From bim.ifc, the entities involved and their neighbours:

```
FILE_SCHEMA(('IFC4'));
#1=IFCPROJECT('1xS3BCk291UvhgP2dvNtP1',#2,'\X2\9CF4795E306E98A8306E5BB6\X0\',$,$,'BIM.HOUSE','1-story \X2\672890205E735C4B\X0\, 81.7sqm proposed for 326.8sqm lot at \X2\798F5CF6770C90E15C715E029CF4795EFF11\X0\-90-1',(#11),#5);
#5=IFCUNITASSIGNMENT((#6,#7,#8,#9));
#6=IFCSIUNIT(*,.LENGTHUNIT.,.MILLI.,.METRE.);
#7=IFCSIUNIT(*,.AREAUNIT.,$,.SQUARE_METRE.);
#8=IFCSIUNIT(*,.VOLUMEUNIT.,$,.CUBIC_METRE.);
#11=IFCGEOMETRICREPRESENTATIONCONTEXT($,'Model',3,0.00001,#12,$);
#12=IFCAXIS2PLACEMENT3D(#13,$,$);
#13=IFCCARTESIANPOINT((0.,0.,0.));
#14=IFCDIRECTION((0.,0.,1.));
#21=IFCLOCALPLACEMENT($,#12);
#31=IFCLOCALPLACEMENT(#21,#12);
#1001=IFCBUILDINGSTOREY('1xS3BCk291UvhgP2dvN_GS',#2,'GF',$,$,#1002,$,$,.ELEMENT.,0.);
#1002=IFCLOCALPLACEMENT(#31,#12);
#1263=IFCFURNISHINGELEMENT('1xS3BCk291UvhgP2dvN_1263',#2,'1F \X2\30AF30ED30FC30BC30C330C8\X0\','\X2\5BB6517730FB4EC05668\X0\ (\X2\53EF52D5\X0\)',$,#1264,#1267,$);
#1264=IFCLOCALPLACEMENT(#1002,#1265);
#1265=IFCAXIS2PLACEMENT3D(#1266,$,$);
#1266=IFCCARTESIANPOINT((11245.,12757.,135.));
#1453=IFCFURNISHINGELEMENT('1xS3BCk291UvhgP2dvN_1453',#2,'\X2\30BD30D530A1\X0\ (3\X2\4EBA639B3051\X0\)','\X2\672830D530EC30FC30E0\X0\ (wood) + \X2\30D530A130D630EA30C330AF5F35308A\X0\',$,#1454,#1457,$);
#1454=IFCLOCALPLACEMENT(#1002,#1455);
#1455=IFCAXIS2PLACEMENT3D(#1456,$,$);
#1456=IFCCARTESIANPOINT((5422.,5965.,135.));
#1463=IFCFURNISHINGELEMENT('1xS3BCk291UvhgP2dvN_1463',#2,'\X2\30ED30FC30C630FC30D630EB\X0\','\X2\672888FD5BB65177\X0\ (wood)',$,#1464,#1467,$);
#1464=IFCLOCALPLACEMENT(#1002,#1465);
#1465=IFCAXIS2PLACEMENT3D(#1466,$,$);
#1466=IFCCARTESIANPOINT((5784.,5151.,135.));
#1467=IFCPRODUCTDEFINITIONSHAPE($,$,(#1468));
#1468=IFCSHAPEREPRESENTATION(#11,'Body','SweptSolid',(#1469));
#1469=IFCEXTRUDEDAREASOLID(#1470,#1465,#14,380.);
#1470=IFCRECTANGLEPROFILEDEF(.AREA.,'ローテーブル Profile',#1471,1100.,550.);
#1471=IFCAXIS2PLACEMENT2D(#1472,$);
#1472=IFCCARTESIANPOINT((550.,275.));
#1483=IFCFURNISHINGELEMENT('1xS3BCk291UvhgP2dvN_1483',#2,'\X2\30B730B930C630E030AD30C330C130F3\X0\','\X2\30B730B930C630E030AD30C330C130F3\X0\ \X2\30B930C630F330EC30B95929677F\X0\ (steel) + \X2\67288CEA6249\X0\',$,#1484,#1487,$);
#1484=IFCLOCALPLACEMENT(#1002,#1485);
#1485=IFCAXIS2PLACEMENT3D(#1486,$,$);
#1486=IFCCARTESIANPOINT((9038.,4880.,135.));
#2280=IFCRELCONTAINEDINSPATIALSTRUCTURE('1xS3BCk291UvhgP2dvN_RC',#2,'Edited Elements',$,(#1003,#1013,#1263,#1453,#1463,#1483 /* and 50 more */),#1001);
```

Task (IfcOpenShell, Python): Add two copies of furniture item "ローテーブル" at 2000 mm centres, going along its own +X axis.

```python
import ifcopenshell
import ifcopenshell.api.geometry
import ifcopenshell.api.root
import ifcopenshell.util.element
import ifcopenshell.util.placement

model = ifcopenshell.open("bim.ifc")


def reuse_history(source, copy):
    """copy_class also copies each property set's owner history, people and application; keep the originals."""
    for rel in copy.IsDefinedBy:
        if rel.is_a("IfcRelDefinesByProperties") and (history := rel.RelatingPropertyDefinition.OwnerHistory):
            rel.RelatingPropertyDefinition.OwnerHistory = source.OwnerHistory
            ifcopenshell.util.element.remove_deep2(model, history)


source = model.by_guid("1xS3BCk291UvhgP2dvN_1463")
base = ifcopenshell.util.placement.get_local_placement(source.ObjectPlacement)
step = base[:3, 0] * 2000.0

for i in range(1, 3):
    copy = ifcopenshell.api.root.copy_class(model, product=source)
    copy.Representation = ifcopenshell.util.element.copy_deep(
        model, source.Representation, exclude=["IfcGeometricRepresentationContext", "IfcRepresentationMap"]
    )
    reuse_history(source, copy)
    matrix = base.copy()
    matrix[:3, 3] += i * step
    print("added at", matrix[:3, 3].round(3) + 0.0)
    ifcopenshell.api.geometry.edit_object_placement(model, product=copy, matrix=matrix, is_si=False)

model.write("bim_v2.ifc")
```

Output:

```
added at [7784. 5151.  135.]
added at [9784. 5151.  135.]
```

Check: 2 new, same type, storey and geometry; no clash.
